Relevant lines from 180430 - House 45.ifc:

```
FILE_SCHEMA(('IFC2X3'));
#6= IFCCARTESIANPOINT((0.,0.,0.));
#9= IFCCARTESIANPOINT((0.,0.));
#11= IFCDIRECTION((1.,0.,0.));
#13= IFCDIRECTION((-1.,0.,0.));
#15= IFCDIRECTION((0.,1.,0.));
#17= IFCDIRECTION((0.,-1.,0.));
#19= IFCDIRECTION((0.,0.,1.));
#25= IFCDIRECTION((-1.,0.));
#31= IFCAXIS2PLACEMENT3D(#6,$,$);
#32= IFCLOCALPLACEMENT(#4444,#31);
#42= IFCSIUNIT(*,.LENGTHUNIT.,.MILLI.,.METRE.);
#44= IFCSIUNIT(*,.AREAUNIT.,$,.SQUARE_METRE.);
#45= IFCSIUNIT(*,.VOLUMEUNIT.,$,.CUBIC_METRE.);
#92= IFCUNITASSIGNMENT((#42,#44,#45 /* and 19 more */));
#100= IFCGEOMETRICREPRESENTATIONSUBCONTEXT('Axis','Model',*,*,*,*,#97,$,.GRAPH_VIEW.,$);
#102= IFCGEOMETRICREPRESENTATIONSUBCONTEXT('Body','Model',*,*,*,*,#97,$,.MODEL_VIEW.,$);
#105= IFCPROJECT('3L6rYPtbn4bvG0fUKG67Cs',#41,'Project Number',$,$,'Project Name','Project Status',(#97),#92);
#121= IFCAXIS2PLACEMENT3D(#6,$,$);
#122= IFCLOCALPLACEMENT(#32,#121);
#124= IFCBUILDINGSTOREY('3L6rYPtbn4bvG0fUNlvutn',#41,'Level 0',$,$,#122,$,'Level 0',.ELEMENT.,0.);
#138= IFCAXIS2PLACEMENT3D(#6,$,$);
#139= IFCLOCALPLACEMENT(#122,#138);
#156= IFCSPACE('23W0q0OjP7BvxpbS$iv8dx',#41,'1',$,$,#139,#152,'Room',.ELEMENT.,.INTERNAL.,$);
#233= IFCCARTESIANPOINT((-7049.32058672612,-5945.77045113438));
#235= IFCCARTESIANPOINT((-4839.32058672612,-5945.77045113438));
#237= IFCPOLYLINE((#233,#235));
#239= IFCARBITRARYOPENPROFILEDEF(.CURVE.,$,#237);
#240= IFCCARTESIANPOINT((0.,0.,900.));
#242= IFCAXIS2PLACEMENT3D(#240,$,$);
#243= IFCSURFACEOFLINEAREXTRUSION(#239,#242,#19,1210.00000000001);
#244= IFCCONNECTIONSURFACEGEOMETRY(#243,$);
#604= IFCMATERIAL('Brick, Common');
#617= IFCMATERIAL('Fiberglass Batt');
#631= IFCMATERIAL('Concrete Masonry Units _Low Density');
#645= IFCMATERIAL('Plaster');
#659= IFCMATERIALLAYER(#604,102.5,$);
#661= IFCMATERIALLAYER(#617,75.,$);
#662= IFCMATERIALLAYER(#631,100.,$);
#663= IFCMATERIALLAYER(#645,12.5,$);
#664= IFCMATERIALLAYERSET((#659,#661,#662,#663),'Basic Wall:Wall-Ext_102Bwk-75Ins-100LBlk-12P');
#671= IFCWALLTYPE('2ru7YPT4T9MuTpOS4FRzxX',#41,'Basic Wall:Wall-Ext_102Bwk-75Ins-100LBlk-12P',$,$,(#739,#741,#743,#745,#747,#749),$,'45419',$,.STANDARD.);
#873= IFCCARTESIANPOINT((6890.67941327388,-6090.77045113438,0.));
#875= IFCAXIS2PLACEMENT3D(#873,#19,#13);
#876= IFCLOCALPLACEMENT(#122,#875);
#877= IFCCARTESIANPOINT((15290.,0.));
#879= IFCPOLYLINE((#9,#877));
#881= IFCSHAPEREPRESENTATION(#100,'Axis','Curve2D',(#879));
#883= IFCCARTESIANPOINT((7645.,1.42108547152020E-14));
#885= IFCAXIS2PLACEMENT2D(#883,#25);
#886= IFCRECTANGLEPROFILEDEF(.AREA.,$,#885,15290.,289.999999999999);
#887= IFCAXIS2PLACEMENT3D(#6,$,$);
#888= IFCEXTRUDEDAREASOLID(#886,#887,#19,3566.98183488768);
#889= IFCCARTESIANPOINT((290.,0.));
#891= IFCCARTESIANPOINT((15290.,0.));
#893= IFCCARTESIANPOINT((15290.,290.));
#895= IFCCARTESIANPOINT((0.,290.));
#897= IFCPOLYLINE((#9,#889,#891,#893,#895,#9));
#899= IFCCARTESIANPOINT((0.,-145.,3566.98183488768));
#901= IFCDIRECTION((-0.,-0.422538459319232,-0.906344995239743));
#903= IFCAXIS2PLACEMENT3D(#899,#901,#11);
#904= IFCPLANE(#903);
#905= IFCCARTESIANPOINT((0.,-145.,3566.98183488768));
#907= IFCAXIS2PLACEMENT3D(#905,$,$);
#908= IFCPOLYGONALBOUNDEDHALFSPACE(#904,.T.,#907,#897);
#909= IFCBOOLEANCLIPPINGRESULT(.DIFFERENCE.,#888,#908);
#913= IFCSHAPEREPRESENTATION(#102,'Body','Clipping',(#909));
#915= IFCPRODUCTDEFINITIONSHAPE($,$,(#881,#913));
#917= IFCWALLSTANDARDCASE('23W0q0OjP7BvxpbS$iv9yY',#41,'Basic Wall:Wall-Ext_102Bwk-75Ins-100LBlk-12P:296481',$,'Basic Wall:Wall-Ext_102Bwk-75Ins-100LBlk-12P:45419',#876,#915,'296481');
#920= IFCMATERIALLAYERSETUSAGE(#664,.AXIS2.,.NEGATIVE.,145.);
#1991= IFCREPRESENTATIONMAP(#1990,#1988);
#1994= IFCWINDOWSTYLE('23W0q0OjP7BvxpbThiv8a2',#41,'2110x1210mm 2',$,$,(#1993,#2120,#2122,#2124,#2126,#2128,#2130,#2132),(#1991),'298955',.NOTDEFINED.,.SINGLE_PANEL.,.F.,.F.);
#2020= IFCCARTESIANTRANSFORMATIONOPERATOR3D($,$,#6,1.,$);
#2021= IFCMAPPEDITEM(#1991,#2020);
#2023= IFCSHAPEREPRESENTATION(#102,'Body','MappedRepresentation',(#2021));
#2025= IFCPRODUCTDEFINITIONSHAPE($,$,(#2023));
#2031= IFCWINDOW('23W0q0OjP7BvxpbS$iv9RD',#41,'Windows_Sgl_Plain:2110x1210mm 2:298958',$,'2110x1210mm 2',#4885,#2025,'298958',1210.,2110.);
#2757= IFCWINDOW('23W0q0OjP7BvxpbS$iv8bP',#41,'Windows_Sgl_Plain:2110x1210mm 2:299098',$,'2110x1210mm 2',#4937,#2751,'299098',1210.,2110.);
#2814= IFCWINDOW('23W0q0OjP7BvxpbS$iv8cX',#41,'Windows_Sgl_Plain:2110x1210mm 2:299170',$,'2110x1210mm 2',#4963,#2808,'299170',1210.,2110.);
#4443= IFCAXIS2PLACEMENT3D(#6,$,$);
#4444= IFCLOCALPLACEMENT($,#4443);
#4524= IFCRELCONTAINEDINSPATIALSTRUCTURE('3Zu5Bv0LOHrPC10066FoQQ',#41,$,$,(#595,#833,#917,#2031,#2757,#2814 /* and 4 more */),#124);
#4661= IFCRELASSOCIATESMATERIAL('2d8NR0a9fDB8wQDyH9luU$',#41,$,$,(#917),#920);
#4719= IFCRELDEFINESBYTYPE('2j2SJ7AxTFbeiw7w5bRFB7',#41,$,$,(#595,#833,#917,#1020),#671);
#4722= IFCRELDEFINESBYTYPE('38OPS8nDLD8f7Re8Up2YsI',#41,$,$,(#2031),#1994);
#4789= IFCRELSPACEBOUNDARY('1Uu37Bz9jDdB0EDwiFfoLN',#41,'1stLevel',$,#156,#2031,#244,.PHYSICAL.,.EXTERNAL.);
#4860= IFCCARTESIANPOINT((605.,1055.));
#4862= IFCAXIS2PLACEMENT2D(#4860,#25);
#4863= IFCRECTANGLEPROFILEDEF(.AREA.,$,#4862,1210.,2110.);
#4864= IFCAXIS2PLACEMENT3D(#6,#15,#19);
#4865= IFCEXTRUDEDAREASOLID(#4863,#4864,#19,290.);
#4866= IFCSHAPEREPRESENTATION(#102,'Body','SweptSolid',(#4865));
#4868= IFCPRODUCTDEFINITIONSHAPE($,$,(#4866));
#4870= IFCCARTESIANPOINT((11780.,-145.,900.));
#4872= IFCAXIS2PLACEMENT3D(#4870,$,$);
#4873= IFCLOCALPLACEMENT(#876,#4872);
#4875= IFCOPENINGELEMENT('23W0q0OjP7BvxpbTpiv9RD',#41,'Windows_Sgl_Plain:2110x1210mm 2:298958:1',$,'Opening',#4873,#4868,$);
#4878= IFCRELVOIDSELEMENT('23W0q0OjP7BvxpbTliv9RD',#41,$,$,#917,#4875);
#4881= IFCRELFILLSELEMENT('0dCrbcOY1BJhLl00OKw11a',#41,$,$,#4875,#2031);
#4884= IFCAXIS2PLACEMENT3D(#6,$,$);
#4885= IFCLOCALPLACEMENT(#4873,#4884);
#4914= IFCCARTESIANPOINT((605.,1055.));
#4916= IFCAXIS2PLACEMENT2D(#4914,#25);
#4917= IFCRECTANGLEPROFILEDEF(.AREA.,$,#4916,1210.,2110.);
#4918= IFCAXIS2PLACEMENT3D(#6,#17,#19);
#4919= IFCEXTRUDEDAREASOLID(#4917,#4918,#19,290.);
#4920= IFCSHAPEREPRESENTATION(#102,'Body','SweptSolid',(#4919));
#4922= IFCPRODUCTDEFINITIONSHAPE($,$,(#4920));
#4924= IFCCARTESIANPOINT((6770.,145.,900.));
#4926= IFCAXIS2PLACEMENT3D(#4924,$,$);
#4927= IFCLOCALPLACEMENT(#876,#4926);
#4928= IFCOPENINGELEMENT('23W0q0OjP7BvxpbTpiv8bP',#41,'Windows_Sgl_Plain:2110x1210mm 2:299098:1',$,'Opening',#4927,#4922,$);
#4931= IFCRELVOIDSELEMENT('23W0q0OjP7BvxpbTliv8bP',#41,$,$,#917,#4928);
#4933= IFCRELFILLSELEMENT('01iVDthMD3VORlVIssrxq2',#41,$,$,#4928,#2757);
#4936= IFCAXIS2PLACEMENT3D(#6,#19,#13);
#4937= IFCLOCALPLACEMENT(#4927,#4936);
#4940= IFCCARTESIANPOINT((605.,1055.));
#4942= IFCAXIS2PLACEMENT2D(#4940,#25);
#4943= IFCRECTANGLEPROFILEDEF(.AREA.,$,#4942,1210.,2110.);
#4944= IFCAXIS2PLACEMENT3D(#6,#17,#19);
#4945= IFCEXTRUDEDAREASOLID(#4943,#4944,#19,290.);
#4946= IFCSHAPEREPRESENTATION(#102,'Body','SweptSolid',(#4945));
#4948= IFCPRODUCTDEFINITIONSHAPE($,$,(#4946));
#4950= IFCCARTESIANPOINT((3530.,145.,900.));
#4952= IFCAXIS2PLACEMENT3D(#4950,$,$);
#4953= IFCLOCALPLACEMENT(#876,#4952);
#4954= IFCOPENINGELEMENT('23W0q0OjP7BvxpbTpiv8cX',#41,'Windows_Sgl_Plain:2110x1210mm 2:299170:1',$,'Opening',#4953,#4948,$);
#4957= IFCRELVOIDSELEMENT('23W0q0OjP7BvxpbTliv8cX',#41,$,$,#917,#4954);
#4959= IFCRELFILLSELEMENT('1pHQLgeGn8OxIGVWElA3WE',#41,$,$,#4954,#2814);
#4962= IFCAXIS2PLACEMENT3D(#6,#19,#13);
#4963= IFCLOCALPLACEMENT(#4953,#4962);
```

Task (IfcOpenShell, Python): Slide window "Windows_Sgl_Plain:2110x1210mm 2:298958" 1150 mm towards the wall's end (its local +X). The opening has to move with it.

```python
import numpy as np
import ifcopenshell
import ifcopenshell.api.geometry
import ifcopenshell.util.placement
import ifcopenshell.util.unit

model = ifcopenshell.open("180430 - House 45.ifc")
unit_scale = ifcopenshell.util.unit.calculate_unit_scale(model)

window = model.by_id(2031)
opening = window.FillsVoids[0].RelatingOpeningElement
wall = opening.VoidsElements[0].RelatingBuildingElement

wall_matrix = ifcopenshell.util.placement.get_local_placement(wall.ObjectPlacement)
shift = wall_matrix[:3, 0] * 1.15 / unit_scale
before = ifcopenshell.util.placement.get_local_placement(window.ObjectPlacement)[:3, 3].copy()

# The window is placed relative to its opening, so it follows when the opening moves.
matrix = ifcopenshell.util.placement.get_local_placement(opening.ObjectPlacement)
matrix[:3, 3] += shift
ifcopenshell.api.geometry.edit_object_placement(
    model, product=opening, matrix=matrix, is_si=False, should_transform_children=True
)

# Space boundary surfaces are stored in each space's coordinates; move them too.
for rel in window.ProvidesBoundaries:
    if not rel.ConnectionGeometry:
        continue
    surface = rel.ConnectionGeometry.SurfaceOnRelatingElement
    space_matrix = ifcopenshell.util.placement.get_local_placement(rel.RelatingSpace.ObjectPlacement)
    point = np.array(surface.Position.Location.Coordinates) + space_matrix[:3, :3].T @ shift
    surface.Position = model.createIfcAxis2Placement3D(
        model.createIfcCartesianPoint(point.tolist()), surface.Position.Axis, surface.Position.RefDirection
    )

after = ifcopenshell.util.placement.get_local_placement(window.ObjectPlacement)[:3, 3]
print("window moved by", (after - before).round(3) + 0.0)

model.write("180430 - House 45_rev.ifc")
```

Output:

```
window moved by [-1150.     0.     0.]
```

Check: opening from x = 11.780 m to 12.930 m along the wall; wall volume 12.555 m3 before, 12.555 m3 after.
